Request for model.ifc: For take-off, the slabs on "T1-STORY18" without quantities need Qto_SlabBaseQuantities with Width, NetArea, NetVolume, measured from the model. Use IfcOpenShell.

First a look at what the model holds.

```python
import ifcopenshell
import ifcopenshell.util.element
import ifcopenshell.util.unit

model = ifcopenshell.open("model.ifc")
print(model.schema)
for unit_type in ("LENGTHUNIT", "AREAUNIT", "VOLUMEUNIT"):
    print(unit_type, ifcopenshell.util.unit.calculate_unit_scale(model, unit_type))
storey = next(s for s in model.by_type("IfcBuildingStorey") if s.Name == "T1-STORY18")
slabs = [e for e in ifcopenshell.util.element.get_decomposition(storey) if e.is_a("IfcSlab")]
for e in sorted(slabs, key=lambda e: e.id()):
    print(e.id(), e.is_a(), e.Name, list(ifcopenshell.util.element.get_psets(e, qtos_only=True)), sep=" | ")
```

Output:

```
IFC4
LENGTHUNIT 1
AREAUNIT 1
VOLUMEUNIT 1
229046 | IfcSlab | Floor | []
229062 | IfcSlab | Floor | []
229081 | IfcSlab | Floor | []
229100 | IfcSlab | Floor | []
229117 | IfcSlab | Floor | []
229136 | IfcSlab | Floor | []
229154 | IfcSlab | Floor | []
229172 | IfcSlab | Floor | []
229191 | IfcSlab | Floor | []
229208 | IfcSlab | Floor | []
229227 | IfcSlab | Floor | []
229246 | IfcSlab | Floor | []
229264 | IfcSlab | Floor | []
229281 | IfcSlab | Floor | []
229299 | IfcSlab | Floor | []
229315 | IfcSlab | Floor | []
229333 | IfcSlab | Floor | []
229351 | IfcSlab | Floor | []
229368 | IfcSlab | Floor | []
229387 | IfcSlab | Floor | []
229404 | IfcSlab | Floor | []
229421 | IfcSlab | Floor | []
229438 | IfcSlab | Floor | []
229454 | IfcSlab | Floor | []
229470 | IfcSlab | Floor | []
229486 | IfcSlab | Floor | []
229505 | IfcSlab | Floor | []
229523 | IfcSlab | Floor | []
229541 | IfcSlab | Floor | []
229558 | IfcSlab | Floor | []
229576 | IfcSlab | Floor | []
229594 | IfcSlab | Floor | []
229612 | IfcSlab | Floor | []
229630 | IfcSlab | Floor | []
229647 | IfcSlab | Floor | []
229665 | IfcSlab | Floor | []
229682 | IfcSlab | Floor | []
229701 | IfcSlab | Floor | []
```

```python
import ifcopenshell
import ifcopenshell.api.pset
import ifcopenshell.geom
import ifcopenshell.util.element
import ifcopenshell.util.shape
import ifcopenshell.util.unit

model = ifcopenshell.open("model.ifc")
unit_scale = ifcopenshell.util.unit.calculate_unit_scale(model)
area_scale = ifcopenshell.util.unit.calculate_unit_scale(model, "AREAUNIT")
volume_scale = ifcopenshell.util.unit.calculate_unit_scale(model, "VOLUMEUNIT")
settings = ifcopenshell.geom.settings()

storey = next(s for s in model.by_type("IfcBuildingStorey") if s.Name == "T1-STORY18")
slabs = [e for e in ifcopenshell.util.element.get_decomposition(storey) if e.is_a("IfcSlab")]

for e in sorted(slabs, key=lambda e: e.id()):
    if ifcopenshell.util.element.get_psets(e, qtos_only=True, should_inherit=False):
        continue
    # Geometry comes back in metres, in the element's own axes.
    shape = ifcopenshell.geom.create_shape(settings, e)
    values = {
        "Width": ifcopenshell.util.shape.get_z(shape.geometry) / unit_scale,
        "NetArea": ifcopenshell.util.shape.get_footprint_area(shape.geometry) / area_scale,
        "NetVolume": ifcopenshell.util.shape.get_volume(shape.geometry) / volume_scale,
    }
    qto = ifcopenshell.api.pset.add_qto(model, product=e, name="Qto_SlabBaseQuantities")
    ifcopenshell.api.pset.edit_qto(model, qto=qto, properties=values)
    print(e.id(), {k: round(v, 3) for k, v in values.items()})

model.write("model_rev.ifc")
```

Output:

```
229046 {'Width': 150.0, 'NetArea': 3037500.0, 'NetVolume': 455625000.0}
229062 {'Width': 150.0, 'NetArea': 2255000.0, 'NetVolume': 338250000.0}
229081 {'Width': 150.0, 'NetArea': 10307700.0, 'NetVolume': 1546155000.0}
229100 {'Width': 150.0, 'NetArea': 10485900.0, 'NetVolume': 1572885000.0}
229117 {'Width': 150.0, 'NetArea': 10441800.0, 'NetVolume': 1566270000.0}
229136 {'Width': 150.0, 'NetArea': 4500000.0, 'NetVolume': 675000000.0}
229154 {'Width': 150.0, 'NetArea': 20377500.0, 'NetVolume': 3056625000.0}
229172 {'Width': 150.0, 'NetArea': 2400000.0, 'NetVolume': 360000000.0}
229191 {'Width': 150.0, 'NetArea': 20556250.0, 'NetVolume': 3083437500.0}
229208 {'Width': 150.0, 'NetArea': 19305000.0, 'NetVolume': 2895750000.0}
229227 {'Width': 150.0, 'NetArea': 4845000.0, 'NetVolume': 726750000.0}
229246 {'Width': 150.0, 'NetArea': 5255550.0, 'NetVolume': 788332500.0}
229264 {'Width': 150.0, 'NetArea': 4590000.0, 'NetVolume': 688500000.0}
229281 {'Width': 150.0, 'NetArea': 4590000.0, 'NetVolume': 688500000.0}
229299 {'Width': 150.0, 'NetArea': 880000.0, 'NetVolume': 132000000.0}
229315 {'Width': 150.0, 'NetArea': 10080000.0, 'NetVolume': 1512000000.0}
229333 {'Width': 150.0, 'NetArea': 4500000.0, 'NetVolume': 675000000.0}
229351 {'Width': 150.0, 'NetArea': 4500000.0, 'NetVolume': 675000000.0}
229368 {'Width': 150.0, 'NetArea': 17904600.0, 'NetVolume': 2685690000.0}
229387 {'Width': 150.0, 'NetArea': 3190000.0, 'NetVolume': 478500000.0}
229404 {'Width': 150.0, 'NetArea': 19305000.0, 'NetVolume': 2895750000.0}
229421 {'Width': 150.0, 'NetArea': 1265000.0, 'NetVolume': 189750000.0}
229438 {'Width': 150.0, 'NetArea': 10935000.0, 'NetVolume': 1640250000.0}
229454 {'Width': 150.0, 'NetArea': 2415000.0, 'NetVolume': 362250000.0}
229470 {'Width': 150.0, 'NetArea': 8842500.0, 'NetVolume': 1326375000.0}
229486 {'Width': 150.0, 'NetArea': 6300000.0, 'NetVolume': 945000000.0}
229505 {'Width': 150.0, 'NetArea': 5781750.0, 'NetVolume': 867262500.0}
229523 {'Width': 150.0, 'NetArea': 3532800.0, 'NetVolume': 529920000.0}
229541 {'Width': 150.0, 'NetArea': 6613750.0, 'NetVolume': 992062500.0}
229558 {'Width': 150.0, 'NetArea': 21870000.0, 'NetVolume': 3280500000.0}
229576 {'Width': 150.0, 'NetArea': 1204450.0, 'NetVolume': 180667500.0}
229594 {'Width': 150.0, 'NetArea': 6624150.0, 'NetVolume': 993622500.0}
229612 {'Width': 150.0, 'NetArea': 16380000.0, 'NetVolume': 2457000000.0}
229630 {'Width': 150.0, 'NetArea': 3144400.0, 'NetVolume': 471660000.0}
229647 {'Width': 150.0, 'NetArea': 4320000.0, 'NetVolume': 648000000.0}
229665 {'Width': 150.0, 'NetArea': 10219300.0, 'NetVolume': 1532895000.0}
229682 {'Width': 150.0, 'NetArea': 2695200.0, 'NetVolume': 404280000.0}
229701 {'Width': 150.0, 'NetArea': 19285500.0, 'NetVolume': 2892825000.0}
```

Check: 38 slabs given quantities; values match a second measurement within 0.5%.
